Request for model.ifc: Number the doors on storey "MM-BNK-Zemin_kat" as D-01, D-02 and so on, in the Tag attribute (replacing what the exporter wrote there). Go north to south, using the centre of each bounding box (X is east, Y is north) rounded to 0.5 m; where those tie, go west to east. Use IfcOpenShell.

First a look at what the model holds.

```python
import ifcopenshell
import ifcopenshell.util.element
import ifcopenshell.util.placement

model = ifcopenshell.open("model.ifc")
print(model.schema)
storey = next(s for s in model.by_type("IfcBuildingStorey") if s.Name == "MM-BNK-Zemin_kat")
doors = [e for e in ifcopenshell.util.element.get_decomposition(storey) if e.is_a("IfcDoor")]
for e in sorted(doors, key=lambda e: e.id()):
    origin = ifcopenshell.util.placement.get_local_placement(e.ObjectPlacement)[:3, 3]
    print(e.id(), e.Tag, e.Name, origin.round(2) + 0.0, sep=" | ")
```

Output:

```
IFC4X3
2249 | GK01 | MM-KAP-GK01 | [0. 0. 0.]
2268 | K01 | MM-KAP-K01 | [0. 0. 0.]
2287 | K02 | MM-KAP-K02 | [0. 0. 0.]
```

```python
import ifcopenshell
import ifcopenshell.geom
import ifcopenshell.util.element
import ifcopenshell.util.shape

model = ifcopenshell.open("model.ifc")
settings = ifcopenshell.geom.settings()
settings.set("use-world-coords", True)


def centre(element):
    shape = ifcopenshell.geom.create_shape(settings, element)
    return ifcopenshell.util.shape.get_bbox_centroid(shape.geometry)


storey = next(s for s in model.by_type("IfcBuildingStorey") if s.Name == "MM-BNK-Zemin_kat")
doors = [e for e in ifcopenshell.util.element.get_decomposition(storey) if e.is_a("IfcDoor")]

# Insertion points can sit at a corner or the storey origin, so sort by the geometry (in metres).
centres = {e: centre(e) for e in doors}
doors.sort(key=lambda e: (-round(centres[e][1] / 0.5), centres[e][0]))

for i, e in enumerate(doors, start=1):
    number = f"D-{i:02d}"
    e.Tag = number
    print(e.id(), number)

model.write("model_rev.ifc")
```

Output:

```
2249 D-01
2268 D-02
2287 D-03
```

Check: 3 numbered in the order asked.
